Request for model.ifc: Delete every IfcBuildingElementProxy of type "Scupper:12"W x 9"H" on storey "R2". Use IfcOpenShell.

First a look at what the model holds.

```python
import ifcopenshell
import ifcopenshell.util.element

model = ifcopenshell.open("model.ifc")
print(model.schema)
storey = next(s for s in model.by_type("IfcBuildingStorey") if s.Name == "R2")
proxies = [e for e in ifcopenshell.util.element.get_decomposition(storey) if e.is_a("IfcBuildingElementProxy")]
seen = {}
for e in proxies:
    element_type = ifcopenshell.util.element.get_type(e)
    name = element_type.Name if element_type not in (None, e) else None
    seen[name] = seen.get(name, 0) + 1
for name, count in sorted(seen.items(), key=str):
    print(count, "x", name)
```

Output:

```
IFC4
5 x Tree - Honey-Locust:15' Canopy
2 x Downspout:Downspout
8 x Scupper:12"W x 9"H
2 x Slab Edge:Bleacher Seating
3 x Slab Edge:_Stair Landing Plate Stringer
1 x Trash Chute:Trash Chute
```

```python
import ifcopenshell
import ifcopenshell.api.root
import ifcopenshell.util.element

model = ifcopenshell.open("model.ifc")

storey = next(s for s in model.by_type("IfcBuildingStorey") if s.Name == "R2")
proxies = [e for e in ifcopenshell.util.element.get_decomposition(storey) if e.is_a("IfcBuildingElementProxy")]
targets = [e for e in proxies if (t := ifcopenshell.util.element.get_type(e)) not in (None, e) and t.Name == 'Scupper:12"W x 9"H']

for e in targets:
    ifcopenshell.api.root.remove_product(model, product=e)
print(len(targets), "removed")

model.write("model_updated.ifc")
```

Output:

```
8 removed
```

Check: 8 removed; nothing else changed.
